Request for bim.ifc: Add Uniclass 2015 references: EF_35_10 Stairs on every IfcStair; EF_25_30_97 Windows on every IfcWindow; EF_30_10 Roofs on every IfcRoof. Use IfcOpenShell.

First a look at what the model holds.

```python
import ifcopenshell

model = ifcopenshell.open("bim.ifc")
print(model.schema)
print("classifications:", [c.Name for c in model.by_type("IfcClassification")])
for ifc_class in ("IfcDoor", "IfcRoof", "IfcStair", "IfcWall", "IfcWindow"):
    print(ifc_class, len(model.by_type(ifc_class)))
```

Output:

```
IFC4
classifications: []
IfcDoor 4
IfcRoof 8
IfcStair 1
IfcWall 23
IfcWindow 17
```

```python
import ifcopenshell
import ifcopenshell.api.classification

model = ifcopenshell.open("bim.ifc")

system = ifcopenshell.api.classification.add_classification(model, classification="Uniclass 2015")

codes = {
    "IfcStair": ("EF_35_10", "Stairs"),
    "IfcWindow": ("EF_25_30_97", "Windows"),
    "IfcRoof": ("EF_30_10", "Roofs"),
}
for ifc_class, (code, name) in codes.items():
    products = model.by_type(ifc_class)
    ifcopenshell.api.classification.add_reference(
        model, products=products, classification=system, identification=code, name=name
    )
    print(code, len(products))

model.write("bim_v2.ifc")
```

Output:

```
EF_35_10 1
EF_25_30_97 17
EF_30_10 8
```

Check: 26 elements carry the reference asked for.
